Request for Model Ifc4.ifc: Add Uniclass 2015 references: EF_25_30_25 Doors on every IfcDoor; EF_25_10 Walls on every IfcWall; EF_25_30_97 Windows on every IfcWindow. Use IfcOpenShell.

First a look at what the model holds.

```python
import ifcopenshell

model = ifcopenshell.open("Model Ifc4.ifc")
print(model.schema)
print("classifications:", [c.Name for c in model.by_type("IfcClassification")])
for ifc_class in ("IfcDoor", "IfcRoof", "IfcStair", "IfcWall", "IfcWindow"):
    print(ifc_class, len(model.by_type(ifc_class)))
```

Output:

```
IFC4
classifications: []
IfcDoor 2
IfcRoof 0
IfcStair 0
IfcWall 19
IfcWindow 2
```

```python
import ifcopenshell
import ifcopenshell.api.classification

model = ifcopenshell.open("Model Ifc4.ifc")

system = ifcopenshell.api.classification.add_classification(model, classification="Uniclass 2015")

codes = {
    "IfcDoor": ("EF_25_30_25", "Doors"),
    "IfcWall": ("EF_25_10", "Walls"),
    "IfcWindow": ("EF_25_30_97", "Windows"),
}
for ifc_class, (code, name) in codes.items():
    products = model.by_type(ifc_class)
    ifcopenshell.api.classification.add_reference(
        model, products=products, classification=system, identification=code, name=name
    )
    print(code, len(products))

model.write("Model Ifc4_v2.ifc")
```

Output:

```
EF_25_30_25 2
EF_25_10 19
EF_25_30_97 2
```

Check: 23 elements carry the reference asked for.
